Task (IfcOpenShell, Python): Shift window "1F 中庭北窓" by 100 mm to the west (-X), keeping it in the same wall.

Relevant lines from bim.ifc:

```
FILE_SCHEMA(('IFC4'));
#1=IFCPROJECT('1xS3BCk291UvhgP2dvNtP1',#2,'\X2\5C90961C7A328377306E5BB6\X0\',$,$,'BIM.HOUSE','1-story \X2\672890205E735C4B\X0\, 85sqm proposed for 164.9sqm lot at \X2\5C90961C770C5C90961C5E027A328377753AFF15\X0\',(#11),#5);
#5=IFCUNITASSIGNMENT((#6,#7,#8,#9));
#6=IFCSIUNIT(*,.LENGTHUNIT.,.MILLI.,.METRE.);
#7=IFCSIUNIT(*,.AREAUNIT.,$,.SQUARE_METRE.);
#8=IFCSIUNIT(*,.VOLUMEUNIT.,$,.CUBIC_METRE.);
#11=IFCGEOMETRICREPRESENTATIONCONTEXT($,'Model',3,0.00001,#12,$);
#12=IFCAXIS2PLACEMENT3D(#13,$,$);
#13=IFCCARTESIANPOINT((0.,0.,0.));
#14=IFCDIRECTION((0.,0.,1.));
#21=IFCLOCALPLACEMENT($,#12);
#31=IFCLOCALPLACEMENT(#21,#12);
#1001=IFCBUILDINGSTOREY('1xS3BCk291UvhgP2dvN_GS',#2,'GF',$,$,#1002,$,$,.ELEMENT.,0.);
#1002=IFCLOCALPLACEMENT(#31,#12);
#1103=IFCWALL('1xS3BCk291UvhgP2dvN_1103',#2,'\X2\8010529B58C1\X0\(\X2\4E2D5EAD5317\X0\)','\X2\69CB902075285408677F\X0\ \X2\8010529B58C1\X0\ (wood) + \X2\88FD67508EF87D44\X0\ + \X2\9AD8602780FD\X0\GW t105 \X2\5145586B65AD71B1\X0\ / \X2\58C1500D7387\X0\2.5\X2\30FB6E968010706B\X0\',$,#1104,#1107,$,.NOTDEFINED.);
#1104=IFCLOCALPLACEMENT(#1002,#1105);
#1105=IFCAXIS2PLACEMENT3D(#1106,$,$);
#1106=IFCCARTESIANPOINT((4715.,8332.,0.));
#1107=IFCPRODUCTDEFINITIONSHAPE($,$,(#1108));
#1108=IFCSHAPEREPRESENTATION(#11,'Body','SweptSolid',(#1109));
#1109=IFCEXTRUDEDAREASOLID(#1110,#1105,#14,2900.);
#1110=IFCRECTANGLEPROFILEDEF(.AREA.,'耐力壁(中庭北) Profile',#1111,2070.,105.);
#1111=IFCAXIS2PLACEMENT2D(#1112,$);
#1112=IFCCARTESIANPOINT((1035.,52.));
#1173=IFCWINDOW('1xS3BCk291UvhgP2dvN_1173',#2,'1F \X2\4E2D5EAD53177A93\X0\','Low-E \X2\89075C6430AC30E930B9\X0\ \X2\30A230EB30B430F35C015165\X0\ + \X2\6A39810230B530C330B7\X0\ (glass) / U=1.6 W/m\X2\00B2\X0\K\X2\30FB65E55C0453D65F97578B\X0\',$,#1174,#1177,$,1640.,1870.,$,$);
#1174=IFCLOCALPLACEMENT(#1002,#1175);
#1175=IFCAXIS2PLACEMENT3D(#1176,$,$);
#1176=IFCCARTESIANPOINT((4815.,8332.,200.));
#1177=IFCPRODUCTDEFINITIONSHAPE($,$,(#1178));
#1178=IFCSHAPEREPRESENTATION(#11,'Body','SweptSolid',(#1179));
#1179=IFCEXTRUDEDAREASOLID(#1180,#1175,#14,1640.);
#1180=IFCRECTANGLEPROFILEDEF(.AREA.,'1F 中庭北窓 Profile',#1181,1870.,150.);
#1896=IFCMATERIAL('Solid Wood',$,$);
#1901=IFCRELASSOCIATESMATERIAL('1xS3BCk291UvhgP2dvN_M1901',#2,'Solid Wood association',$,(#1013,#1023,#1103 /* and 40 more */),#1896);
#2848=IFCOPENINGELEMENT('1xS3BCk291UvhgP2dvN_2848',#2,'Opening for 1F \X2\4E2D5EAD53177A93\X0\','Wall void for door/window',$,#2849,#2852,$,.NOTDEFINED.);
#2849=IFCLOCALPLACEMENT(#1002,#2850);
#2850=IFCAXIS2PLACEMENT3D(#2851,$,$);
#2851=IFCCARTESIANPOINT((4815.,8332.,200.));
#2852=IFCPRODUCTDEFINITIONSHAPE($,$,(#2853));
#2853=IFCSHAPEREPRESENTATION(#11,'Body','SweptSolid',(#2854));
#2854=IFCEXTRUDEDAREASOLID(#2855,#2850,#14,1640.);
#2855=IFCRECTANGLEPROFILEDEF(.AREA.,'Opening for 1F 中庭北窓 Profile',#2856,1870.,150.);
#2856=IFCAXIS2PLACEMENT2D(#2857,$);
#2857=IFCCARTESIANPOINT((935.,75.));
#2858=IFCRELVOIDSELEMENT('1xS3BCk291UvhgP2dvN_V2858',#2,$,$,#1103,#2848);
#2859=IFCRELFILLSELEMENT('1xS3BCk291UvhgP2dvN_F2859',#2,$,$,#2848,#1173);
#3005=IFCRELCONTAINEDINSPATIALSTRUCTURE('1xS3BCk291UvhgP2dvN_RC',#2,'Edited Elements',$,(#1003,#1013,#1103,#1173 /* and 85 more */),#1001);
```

```python
import ifcopenshell
import ifcopenshell.api.geometry
import ifcopenshell.util.placement
import ifcopenshell.util.unit

model = ifcopenshell.open("bim.ifc")
unit_scale = ifcopenshell.util.unit.calculate_unit_scale(model)

window = model.by_id(1173)
opening = window.FillsVoids[0].RelatingOpeningElement
wall = opening.VoidsElements[0].RelatingBuildingElement

wall_matrix = ifcopenshell.util.placement.get_local_placement(wall.ObjectPlacement)
shift = wall_matrix[:3, 0] * -0.1 / unit_scale
before = ifcopenshell.util.placement.get_local_placement(window.ObjectPlacement)[:3, 3].copy()

# The window is not placed relative to its opening, so move both.
for product in (opening, window):
    matrix = ifcopenshell.util.placement.get_local_placement(product.ObjectPlacement)
    matrix[:3, 3] += shift
    ifcopenshell.api.geometry.edit_object_placement(model, product=product, matrix=matrix, is_si=False)

after = ifcopenshell.util.placement.get_local_placement(window.ObjectPlacement)[:3, 3]
print("window moved by", (after - before).round(3) + 0.0)

model.write("bim_edited.ifc")
```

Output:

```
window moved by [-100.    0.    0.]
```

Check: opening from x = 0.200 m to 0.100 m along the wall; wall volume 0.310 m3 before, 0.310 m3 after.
